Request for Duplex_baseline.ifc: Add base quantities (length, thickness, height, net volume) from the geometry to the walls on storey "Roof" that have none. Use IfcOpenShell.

First a look at what the model holds.

```python
import ifcopenshell
import ifcopenshell.util.element
import ifcopenshell.util.unit

model = ifcopenshell.open("Duplex_baseline.ifc")
print(model.schema)
for unit_type in ("LENGTHUNIT", "AREAUNIT", "VOLUMEUNIT"):
    print(unit_type, ifcopenshell.util.unit.calculate_unit_scale(model, unit_type))
storey = next(s for s in model.by_type("IfcBuildingStorey") if s.Name == "Roof")
walls = [e for e in ifcopenshell.util.element.get_decomposition(storey) if e.is_a("IfcWall")]
for e in sorted(walls, key=lambda e: e.id()):
    print(e.id(), e.is_a(), e.Name, list(ifcopenshell.util.element.get_psets(e, qtos_only=True)), sep=" | ")
```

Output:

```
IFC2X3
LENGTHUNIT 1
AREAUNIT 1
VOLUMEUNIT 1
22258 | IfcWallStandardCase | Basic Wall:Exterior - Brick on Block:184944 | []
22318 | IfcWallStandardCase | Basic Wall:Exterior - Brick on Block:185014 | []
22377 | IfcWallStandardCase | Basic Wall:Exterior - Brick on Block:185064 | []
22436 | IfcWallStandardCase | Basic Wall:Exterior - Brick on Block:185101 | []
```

```python
import ifcopenshell
import ifcopenshell.api.pset
import ifcopenshell.geom
import ifcopenshell.util.element
import ifcopenshell.util.shape
import ifcopenshell.util.unit

model = ifcopenshell.open("Duplex_baseline.ifc")
unit_scale = ifcopenshell.util.unit.calculate_unit_scale(model)
volume_scale = ifcopenshell.util.unit.calculate_unit_scale(model, "VOLUMEUNIT")
settings = ifcopenshell.geom.settings()

storey = next(s for s in model.by_type("IfcBuildingStorey") if s.Name == "Roof")
walls = [e for e in ifcopenshell.util.element.get_decomposition(storey) if e.is_a("IfcWall")]

for e in sorted(walls, key=lambda e: e.id()):
    if ifcopenshell.util.element.get_psets(e, qtos_only=True, should_inherit=False):
        continue
    # Geometry comes back in metres, in the element's own axes.
    shape = ifcopenshell.geom.create_shape(settings, e)
    values = {
        "Length": ifcopenshell.util.shape.get_x(shape.geometry) / unit_scale,
        "Width": ifcopenshell.util.shape.get_y(shape.geometry) / unit_scale,
        "Height": ifcopenshell.util.shape.get_z(shape.geometry) / unit_scale,
        "NetVolume": ifcopenshell.util.shape.get_volume(shape.geometry) / volume_scale,
    }
    qto = ifcopenshell.api.pset.add_qto(model, product=e, name="BaseQuantities")
    ifcopenshell.api.pset.edit_qto(model, qto=qto, properties=values)
    print(e.id(), {k: round(v, 3) for k, v in values.items()})

model.write("Duplex_baseline_edited.ifc")
```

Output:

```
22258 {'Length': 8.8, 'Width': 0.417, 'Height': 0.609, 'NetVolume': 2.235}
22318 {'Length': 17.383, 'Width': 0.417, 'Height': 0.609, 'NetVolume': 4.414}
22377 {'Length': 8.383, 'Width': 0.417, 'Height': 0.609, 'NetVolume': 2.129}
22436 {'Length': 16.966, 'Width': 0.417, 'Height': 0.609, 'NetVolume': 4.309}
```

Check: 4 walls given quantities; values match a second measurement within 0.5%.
